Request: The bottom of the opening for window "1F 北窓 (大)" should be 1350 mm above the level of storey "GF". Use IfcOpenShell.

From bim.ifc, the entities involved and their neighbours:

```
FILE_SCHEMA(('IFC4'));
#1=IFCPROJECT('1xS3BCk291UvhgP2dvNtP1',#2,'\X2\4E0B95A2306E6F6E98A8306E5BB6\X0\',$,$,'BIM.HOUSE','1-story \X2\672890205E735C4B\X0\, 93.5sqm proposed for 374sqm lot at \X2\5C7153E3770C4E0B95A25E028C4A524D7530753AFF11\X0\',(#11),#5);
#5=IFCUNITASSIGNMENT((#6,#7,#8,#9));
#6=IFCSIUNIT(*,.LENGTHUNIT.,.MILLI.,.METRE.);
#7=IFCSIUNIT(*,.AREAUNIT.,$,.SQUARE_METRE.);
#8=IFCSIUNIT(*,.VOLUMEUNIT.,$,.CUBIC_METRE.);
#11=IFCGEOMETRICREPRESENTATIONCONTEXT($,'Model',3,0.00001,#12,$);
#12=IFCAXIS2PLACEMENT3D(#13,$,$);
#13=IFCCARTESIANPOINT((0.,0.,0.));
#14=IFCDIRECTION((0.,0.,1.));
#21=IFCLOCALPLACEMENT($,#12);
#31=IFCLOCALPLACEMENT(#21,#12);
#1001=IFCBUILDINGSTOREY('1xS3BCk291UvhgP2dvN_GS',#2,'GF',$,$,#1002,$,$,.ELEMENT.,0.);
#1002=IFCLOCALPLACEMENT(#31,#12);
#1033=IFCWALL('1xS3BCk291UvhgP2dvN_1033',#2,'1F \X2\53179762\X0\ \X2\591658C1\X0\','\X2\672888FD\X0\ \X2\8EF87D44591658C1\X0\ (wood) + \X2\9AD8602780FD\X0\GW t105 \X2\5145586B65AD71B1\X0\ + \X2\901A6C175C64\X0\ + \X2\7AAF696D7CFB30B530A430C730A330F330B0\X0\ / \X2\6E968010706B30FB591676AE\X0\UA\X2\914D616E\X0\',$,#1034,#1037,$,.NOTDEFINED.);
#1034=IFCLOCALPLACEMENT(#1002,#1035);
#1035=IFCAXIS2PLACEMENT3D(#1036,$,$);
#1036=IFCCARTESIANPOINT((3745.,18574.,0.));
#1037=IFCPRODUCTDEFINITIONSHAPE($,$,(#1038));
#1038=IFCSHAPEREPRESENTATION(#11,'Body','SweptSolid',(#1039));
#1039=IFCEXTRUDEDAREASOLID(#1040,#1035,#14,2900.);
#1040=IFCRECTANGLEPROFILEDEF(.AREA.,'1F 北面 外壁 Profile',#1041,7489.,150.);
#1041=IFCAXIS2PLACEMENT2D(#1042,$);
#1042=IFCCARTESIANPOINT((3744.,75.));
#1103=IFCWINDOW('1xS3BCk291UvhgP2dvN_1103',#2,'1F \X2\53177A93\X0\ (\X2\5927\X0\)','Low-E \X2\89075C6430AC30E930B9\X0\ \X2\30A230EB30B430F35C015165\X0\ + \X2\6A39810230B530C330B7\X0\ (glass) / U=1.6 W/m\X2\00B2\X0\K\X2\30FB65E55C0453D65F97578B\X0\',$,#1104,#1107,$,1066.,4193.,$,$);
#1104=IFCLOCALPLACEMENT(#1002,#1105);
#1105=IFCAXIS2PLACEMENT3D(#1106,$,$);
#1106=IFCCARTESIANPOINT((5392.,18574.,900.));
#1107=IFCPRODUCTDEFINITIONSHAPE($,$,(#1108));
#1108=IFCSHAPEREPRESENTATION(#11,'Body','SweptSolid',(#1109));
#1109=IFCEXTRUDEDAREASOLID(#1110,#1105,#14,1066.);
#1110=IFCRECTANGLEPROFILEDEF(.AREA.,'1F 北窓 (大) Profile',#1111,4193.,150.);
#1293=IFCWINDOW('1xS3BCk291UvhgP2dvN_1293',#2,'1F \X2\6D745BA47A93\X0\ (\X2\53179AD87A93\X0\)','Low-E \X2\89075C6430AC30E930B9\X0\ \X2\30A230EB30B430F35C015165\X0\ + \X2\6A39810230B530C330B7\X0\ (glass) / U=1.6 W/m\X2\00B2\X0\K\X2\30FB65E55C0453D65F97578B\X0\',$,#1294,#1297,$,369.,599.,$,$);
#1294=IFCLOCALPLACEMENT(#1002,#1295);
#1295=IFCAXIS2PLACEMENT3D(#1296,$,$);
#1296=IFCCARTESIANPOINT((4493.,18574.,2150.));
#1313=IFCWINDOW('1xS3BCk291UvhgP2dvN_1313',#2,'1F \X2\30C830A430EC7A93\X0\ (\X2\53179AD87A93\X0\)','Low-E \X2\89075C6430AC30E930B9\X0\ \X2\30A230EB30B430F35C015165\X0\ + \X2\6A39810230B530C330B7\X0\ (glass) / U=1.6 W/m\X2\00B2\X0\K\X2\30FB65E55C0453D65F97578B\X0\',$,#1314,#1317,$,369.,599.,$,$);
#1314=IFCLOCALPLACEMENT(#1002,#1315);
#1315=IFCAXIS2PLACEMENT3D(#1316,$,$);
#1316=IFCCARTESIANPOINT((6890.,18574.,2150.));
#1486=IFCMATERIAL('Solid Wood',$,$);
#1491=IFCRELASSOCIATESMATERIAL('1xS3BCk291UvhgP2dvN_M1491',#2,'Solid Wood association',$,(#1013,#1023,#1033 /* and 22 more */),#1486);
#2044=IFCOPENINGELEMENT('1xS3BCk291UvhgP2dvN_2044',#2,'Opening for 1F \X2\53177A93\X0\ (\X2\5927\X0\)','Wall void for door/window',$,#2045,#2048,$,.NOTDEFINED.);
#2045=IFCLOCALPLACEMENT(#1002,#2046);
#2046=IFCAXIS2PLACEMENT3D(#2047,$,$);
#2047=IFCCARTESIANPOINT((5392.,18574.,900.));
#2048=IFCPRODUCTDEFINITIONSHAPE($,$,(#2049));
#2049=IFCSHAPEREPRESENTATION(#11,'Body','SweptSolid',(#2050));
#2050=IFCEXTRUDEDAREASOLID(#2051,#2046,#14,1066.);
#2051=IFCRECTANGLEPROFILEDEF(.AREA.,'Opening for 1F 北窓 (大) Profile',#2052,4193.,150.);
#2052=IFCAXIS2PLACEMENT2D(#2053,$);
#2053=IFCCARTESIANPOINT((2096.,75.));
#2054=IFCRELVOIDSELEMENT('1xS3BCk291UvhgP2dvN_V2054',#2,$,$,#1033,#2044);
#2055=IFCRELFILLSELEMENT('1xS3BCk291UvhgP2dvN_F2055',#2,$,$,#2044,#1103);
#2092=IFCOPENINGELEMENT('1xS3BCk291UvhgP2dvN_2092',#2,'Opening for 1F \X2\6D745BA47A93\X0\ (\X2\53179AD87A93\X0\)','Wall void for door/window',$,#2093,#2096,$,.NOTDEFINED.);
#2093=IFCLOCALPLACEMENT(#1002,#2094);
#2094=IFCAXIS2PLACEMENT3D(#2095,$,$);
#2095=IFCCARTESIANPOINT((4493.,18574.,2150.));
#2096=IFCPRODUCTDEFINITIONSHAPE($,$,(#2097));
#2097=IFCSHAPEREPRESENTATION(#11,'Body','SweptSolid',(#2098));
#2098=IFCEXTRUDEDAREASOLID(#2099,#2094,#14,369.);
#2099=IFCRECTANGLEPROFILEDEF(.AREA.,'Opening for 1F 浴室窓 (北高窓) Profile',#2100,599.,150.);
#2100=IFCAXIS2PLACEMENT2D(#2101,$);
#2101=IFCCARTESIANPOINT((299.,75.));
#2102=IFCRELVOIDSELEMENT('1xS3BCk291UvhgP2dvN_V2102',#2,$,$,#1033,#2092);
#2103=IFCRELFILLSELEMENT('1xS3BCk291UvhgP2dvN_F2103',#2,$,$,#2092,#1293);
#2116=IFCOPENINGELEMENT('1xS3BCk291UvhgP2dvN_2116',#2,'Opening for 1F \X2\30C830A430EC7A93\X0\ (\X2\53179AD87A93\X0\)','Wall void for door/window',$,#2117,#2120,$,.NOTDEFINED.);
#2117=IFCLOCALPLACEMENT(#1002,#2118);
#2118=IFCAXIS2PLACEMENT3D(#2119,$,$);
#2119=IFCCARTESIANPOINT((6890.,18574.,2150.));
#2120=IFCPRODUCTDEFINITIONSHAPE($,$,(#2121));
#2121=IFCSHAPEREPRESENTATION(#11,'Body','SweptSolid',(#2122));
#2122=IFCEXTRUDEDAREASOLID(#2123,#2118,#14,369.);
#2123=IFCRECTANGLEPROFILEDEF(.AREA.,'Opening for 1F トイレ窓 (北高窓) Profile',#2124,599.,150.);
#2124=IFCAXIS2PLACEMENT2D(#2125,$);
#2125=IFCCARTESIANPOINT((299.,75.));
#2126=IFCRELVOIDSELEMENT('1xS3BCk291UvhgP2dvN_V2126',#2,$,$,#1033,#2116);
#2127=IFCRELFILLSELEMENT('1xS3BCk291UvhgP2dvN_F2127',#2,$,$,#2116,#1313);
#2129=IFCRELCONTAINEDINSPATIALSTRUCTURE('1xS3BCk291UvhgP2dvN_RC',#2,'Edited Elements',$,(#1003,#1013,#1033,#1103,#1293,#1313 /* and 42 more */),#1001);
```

```python
import numpy as np
import ifcopenshell
import ifcopenshell.api.geometry
import ifcopenshell.geom
import ifcopenshell.util.element
import ifcopenshell.util.placement
import ifcopenshell.util.shape
import ifcopenshell.util.unit

model = ifcopenshell.open("bim.ifc")
unit_scale = ifcopenshell.util.unit.calculate_unit_scale(model)

window = model.by_id(1103)
opening = window.FillsVoids[0].RelatingOpeningElement
storey = ifcopenshell.util.element.get_container(window, ifc_class="IfcBuildingStorey")
level = ifcopenshell.util.placement.get_local_placement(storey.ObjectPlacement)[2, 3]

# The opening's origin need not be at the sill, so measure its lowest point.
shape = ifcopenshell.geom.create_shape(ifcopenshell.geom.settings(), opening)
bottom = ifcopenshell.util.shape.get_shape_bottom_elevation(shape, shape.geometry) / unit_scale
dz = level + 1350.0 - bottom

shift = np.array([0.0, 0.0, dz])
# The window is not placed relative to its opening, so move both.
for product in (opening, window):
    matrix = ifcopenshell.util.placement.get_local_placement(product.ObjectPlacement)
    matrix[:3, 3] += shift
    ifcopenshell.api.geometry.edit_object_placement(model, product=product, matrix=matrix, is_si=False)

print(f"moved by {dz * unit_scale:+.3f} m")

model.write("bim_rev.ifc")
```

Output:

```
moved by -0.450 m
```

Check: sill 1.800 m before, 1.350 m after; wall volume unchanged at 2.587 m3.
